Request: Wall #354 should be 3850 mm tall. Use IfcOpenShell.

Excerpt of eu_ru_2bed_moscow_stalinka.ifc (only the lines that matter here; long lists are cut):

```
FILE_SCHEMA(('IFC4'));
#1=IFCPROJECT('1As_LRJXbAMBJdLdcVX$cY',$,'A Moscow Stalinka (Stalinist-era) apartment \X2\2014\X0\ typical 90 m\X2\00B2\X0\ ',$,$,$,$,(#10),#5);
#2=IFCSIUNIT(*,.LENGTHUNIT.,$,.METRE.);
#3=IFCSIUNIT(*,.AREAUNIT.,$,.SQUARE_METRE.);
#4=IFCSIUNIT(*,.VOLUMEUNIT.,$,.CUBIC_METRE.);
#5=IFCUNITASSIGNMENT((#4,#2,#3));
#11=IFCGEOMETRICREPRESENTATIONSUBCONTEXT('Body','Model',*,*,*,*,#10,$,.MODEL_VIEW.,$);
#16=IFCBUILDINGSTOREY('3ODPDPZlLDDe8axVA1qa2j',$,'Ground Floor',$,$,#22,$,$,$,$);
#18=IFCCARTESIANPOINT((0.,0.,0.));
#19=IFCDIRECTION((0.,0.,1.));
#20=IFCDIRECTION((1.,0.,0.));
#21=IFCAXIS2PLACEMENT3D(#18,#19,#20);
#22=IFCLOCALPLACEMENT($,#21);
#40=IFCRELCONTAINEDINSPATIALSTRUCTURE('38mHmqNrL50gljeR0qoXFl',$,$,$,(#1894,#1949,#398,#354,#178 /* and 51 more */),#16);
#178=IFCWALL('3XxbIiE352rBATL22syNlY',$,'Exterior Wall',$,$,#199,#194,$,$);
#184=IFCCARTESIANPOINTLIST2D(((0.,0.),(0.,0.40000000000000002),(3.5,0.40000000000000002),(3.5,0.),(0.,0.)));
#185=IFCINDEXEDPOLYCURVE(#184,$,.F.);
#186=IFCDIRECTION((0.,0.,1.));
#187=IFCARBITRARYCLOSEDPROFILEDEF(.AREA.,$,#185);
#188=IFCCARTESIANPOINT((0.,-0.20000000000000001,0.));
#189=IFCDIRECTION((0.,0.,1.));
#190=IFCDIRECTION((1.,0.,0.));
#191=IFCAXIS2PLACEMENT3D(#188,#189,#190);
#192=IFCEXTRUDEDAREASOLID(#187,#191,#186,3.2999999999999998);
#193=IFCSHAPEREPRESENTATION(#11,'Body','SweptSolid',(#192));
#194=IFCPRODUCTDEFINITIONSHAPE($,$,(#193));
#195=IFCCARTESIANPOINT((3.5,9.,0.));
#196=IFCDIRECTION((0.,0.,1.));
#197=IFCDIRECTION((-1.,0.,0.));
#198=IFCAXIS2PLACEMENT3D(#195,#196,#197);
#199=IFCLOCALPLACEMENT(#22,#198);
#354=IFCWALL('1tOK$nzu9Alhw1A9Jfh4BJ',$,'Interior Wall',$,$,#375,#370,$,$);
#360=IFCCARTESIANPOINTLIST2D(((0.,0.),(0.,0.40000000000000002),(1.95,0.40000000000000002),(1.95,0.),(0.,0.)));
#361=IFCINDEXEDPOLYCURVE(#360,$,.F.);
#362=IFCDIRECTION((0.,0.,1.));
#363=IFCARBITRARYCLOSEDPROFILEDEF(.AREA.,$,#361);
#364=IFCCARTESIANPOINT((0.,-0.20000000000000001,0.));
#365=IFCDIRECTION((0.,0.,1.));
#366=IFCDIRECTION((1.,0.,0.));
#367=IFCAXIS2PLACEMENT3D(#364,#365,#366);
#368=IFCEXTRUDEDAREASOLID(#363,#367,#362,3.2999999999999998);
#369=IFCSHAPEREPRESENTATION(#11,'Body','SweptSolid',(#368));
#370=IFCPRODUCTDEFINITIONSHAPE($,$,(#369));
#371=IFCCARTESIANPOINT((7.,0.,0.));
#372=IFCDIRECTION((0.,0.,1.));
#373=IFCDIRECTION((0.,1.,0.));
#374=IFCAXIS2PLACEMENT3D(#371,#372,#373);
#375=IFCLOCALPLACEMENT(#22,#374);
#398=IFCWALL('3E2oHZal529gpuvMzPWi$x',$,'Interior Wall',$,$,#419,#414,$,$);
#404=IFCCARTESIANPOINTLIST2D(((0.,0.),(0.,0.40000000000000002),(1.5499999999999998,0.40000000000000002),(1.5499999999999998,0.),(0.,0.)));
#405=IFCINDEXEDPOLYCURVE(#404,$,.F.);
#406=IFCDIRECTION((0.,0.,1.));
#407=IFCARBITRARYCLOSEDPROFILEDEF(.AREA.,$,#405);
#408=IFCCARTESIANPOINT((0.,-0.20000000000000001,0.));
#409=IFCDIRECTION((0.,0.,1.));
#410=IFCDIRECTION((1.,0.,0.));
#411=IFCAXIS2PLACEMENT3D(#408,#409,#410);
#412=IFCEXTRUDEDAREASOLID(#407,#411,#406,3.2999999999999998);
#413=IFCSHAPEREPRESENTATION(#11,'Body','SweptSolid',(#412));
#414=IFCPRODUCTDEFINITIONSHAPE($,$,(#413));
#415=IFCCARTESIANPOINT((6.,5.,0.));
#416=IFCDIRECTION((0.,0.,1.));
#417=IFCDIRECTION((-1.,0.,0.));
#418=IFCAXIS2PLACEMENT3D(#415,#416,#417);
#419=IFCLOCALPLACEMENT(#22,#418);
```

```python
import ifcopenshell
import ifcopenshell.geom
import ifcopenshell.util.representation
import ifcopenshell.util.shape
import ifcopenshell.util.unit

model = ifcopenshell.open("eu_ru_2bed_moscow_stalinka.ifc")
unit_scale = ifcopenshell.util.unit.calculate_unit_scale(model)
settings = ifcopenshell.geom.settings()


def volume(element):
    """Net volume in cubic metres, openings subtracted."""
    shape = ifcopenshell.geom.create_shape(settings, element)
    return ifcopenshell.util.shape.get_volume(shape.geometry)


wall = model.by_guid("1tOK$nzu9Alhw1A9Jfh4BJ")
before = volume(wall)

body = ifcopenshell.util.representation.get_representation(wall, "Model", "Body")
solid = body.Items[0]
old_height = solid.Depth
solid.Depth = 3.85 / unit_scale
after = volume(wall)

print(f"height {old_height:g} -> {solid.Depth:g}, volume {before:.3f} -> {after:.3f} m3")

model.write("eu_ru_2bed_moscow_stalinka_updated.ifc")
```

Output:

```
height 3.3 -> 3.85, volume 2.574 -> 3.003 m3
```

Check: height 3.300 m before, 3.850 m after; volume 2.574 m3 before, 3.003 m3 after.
